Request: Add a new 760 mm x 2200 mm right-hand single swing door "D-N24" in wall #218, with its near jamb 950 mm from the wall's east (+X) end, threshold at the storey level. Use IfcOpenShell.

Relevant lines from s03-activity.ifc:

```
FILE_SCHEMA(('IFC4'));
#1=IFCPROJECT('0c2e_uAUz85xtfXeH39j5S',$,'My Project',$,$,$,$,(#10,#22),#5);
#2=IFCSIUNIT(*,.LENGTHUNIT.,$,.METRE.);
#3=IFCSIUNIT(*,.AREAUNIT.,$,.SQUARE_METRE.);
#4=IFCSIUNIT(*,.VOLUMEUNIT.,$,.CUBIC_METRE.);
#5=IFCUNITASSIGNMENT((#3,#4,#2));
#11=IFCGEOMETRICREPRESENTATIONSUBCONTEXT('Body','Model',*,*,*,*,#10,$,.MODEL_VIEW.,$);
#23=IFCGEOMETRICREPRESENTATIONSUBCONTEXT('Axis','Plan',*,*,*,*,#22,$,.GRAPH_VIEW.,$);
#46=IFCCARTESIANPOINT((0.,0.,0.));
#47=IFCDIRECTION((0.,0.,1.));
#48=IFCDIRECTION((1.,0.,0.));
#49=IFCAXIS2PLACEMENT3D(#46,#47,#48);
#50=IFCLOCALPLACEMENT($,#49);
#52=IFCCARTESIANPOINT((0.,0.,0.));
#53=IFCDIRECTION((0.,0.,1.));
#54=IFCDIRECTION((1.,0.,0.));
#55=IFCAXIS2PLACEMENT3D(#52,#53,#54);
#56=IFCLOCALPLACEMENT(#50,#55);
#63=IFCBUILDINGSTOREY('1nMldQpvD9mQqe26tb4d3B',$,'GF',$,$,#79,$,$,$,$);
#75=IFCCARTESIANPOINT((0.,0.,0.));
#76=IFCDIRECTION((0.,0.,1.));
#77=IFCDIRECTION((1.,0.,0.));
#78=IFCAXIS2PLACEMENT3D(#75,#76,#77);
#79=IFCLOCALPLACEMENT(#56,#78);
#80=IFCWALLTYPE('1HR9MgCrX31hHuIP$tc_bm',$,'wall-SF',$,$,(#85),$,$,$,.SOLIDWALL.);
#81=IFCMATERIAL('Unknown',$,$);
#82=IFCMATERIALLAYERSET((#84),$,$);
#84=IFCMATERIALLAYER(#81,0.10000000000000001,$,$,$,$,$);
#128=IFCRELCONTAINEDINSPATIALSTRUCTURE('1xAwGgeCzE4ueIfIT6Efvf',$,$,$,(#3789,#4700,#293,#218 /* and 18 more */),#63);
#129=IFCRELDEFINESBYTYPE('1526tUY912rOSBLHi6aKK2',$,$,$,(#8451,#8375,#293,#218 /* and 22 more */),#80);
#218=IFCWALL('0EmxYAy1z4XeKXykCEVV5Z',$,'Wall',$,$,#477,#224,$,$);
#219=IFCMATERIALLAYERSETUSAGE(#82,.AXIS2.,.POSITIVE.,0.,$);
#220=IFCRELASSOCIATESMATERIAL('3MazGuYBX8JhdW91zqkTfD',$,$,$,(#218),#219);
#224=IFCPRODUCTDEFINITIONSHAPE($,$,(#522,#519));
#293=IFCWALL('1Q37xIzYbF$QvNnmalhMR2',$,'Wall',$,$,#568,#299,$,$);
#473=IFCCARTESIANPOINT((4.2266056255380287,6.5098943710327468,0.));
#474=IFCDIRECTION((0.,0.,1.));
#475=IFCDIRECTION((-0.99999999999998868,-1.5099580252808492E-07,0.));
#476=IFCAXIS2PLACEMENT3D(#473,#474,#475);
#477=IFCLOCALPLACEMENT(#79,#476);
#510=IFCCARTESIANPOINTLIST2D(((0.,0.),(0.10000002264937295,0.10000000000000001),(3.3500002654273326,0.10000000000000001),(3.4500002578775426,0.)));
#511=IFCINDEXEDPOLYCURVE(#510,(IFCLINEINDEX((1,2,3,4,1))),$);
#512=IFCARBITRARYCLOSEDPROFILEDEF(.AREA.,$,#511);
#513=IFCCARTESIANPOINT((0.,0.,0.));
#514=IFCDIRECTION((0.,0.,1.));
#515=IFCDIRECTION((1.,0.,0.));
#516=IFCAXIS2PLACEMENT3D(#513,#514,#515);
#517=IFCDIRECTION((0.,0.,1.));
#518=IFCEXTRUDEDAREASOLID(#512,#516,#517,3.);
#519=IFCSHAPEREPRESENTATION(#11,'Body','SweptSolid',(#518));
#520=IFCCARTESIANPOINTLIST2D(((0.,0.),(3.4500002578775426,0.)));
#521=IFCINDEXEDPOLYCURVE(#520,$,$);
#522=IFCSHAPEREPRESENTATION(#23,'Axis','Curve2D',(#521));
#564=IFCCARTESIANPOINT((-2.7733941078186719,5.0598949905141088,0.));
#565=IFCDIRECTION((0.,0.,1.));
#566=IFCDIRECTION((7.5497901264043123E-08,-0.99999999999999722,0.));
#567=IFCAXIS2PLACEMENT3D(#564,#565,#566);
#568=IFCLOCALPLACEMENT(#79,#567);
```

```python
import numpy as np
import ifcopenshell
import ifcopenshell.api.feature
import ifcopenshell.api.geometry
import ifcopenshell.api.root
import ifcopenshell.api.spatial
import ifcopenshell.geom
import ifcopenshell.util.element
import ifcopenshell.util.placement
import ifcopenshell.util.representation
import ifcopenshell.util.shape
import ifcopenshell.util.unit

model = ifcopenshell.open("s03-activity.ifc")
unit_scale = ifcopenshell.util.unit.calculate_unit_scale(model)
settings = ifcopenshell.geom.settings()


def volume(element):
    """Net volume in cubic metres, openings subtracted."""
    shape = ifcopenshell.geom.create_shape(settings, element)
    return ifcopenshell.util.shape.get_volume(shape.geometry)


wall = model.by_guid("0EmxYAy1z4XeKXykCEVV5Z")
storey = ifcopenshell.util.element.get_container(wall, ifc_class="IfcBuildingStorey")
context = ifcopenshell.util.representation.get_context(model, "Model", "Body", "MODEL_VIEW")
before = volume(wall)

width, height, from_end, sill = 0.76, 2.2, 0.95, 0.0  # metres

# The wall runs along its own X axis, and the end named is its -X end.
wall_shape = ifcopenshell.geom.create_shape(settings, wall)
x, y, z = ifcopenshell.util.shape.get_vertices(wall_shape.geometry).T
start = x.min() + from_end
face, thickness = float(y.min()), float(y.max() - y.min())
wall_matrix = ifcopenshell.util.placement.get_local_placement(wall.ObjectPlacement)
level = ifcopenshell.util.placement.get_local_placement(storey.ObjectPlacement)[2, 3]


def in_wall(x, y):
    """Placement at x, y metres in the wall's axes, at sill height."""
    matrix = wall_matrix.copy()
    matrix[:, 3] = wall_matrix @ np.array([x / unit_scale, y / unit_scale, 0.0, 1.0])
    matrix[2, 3] = level + sill / unit_scale
    return matrix


# Opening: a box that overshoots both wall faces by 50 mm.
opening = ifcopenshell.api.root.create_entity(model, ifc_class="IfcOpeningElement", predefined_type="OPENING")
box = ifcopenshell.api.geometry.add_wall_representation(
    model, context=context, length=width, height=height, thickness=thickness + 0.1
)
ifcopenshell.api.geometry.assign_representation(model, product=opening, representation=box)
ifcopenshell.api.geometry.edit_object_placement(model, product=opening, matrix=in_wall(start, face - 0.05), is_si=False)
ifcopenshell.api.feature.add_feature(model, feature=opening, element=wall)

door = ifcopenshell.api.root.create_entity(model, ifc_class="IfcDoor", name="D-N24", predefined_type="DOOR")
door.OverallWidth, door.OverallHeight = width / unit_scale, height / unit_scale
door.OperationType = "SINGLE_SWING_RIGHT"
body = ifcopenshell.api.geometry.add_door_representation(
    model,
    context=context,
    overall_width=door.OverallWidth,
    overall_height=door.OverallHeight,
    operation_type="SINGLE_SWING_RIGHT",
    lining_properties={"LiningDepth": thickness / unit_scale, "ThresholdDepth": thickness / unit_scale},
)
ifcopenshell.api.geometry.assign_representation(model, product=door, representation=body)
ifcopenshell.api.spatial.assign_container(model, products=[door], relating_structure=storey)
ifcopenshell.api.feature.add_filling(model, opening=opening, element=door)

# The lining spans the wall, so the door starts at the wall face.
ifcopenshell.api.geometry.edit_object_placement(model, product=door, matrix=in_wall(start, face), is_si=False)

after = volume(wall)

print(f"wall volume {before:.3f} -> {after:.3f} m3")

model.write("s03-activity_rev.ifc")
```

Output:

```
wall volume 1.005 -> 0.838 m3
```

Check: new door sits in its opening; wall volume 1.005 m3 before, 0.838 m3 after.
